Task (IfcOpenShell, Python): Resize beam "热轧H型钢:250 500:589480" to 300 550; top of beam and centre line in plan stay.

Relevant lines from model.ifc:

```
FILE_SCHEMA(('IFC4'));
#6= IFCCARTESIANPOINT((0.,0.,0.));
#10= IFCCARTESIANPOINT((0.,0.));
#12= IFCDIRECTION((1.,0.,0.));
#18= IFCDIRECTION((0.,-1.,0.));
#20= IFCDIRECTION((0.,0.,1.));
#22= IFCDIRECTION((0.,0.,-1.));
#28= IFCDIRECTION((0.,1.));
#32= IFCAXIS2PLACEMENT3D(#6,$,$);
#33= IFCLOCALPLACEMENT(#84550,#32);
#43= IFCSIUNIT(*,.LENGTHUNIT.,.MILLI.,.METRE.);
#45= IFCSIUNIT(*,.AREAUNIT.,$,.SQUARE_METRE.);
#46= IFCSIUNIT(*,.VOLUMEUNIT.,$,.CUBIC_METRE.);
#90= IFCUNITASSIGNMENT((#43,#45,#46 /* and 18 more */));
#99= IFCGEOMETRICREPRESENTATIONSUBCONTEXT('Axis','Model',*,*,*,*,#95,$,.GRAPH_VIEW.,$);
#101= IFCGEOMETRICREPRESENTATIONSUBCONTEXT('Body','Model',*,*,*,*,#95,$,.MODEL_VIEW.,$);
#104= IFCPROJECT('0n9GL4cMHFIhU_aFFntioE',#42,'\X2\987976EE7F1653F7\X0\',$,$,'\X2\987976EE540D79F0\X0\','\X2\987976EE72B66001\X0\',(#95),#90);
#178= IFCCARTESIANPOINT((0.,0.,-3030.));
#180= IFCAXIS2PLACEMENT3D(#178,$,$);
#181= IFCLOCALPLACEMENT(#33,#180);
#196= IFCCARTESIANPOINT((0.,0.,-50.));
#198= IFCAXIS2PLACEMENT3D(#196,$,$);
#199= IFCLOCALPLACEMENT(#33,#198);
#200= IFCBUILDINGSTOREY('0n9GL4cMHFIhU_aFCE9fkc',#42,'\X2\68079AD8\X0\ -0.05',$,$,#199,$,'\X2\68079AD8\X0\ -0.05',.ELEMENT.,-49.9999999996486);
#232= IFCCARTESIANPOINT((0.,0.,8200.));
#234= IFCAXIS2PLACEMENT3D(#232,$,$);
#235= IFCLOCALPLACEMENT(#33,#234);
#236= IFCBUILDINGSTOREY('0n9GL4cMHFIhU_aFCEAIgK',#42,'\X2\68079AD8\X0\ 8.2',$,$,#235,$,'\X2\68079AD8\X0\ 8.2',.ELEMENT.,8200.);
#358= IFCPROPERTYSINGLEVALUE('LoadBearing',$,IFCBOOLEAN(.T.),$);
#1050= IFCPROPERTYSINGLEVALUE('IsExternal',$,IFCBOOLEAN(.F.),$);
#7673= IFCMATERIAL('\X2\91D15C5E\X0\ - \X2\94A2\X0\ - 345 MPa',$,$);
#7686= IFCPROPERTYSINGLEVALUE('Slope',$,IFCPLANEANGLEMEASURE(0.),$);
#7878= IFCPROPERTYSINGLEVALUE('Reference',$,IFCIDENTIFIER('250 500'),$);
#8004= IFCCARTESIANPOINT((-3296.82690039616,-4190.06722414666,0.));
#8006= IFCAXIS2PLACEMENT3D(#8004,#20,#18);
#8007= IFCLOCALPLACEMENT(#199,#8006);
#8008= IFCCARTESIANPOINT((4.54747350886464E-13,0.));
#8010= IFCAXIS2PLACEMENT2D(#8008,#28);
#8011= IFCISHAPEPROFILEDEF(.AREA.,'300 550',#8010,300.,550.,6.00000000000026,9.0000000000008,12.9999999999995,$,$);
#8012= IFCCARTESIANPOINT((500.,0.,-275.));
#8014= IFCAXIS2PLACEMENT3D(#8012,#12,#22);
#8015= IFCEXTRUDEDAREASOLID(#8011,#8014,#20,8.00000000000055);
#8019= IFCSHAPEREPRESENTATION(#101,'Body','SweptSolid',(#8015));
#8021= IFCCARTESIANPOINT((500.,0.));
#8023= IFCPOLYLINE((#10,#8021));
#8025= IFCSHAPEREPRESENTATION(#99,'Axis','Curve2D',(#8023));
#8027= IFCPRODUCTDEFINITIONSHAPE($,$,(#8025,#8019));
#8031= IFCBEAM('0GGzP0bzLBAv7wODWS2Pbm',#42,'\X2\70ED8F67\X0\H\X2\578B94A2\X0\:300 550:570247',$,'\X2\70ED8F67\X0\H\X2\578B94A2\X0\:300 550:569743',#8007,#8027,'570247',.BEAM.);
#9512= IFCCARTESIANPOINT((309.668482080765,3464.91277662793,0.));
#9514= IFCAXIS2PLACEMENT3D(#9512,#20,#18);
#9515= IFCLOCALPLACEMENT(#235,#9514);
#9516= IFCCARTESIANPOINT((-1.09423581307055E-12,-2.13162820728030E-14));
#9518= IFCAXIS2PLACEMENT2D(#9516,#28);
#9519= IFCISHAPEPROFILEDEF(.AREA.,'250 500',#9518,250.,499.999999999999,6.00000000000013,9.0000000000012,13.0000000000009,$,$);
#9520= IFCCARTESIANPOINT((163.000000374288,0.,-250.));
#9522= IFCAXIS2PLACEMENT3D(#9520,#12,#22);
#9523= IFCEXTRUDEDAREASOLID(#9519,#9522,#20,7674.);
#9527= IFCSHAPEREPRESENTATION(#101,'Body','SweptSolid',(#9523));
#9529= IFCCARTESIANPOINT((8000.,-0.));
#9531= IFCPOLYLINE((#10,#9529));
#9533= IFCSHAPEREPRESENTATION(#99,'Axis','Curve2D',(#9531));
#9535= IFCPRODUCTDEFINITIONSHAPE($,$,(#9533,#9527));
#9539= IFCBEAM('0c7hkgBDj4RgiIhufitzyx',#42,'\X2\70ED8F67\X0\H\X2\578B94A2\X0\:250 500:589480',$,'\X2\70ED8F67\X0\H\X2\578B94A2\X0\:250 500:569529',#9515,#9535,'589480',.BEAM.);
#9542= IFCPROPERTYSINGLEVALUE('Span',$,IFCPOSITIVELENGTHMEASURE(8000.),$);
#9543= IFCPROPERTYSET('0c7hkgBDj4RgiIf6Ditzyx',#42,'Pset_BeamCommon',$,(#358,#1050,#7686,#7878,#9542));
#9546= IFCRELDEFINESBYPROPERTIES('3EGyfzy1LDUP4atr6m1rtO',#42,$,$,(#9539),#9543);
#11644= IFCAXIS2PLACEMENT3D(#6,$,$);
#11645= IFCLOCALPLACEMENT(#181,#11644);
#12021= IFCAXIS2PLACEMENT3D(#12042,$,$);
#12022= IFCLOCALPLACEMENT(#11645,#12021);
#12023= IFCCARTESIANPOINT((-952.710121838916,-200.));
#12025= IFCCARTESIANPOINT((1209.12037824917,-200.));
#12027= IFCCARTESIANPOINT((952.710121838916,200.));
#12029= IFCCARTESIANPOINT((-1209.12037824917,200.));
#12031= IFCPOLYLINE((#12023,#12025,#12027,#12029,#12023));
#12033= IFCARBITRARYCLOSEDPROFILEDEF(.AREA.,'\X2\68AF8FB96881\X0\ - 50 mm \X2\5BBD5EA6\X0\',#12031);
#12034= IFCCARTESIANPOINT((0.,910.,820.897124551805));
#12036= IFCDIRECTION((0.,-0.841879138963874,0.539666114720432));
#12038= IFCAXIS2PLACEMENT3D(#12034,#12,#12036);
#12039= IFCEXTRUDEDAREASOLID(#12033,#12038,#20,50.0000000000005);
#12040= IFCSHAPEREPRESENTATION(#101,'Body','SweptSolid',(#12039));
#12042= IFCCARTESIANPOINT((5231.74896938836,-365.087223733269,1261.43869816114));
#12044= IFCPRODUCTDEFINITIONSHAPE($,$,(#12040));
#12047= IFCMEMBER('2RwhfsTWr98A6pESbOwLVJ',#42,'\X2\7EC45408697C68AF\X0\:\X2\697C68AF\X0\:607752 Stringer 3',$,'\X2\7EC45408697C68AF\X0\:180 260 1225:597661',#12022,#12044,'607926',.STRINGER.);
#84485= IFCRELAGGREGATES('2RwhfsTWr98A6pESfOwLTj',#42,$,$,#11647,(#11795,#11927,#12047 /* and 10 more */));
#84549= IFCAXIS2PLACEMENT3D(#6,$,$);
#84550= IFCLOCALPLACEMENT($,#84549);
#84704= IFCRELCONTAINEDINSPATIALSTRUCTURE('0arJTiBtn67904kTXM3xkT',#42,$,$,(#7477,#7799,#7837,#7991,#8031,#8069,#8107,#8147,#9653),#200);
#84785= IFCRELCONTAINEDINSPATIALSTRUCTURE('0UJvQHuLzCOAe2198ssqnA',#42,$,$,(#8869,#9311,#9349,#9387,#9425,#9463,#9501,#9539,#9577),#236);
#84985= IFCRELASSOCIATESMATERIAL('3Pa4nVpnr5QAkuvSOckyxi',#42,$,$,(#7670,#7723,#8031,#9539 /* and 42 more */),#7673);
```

```python
import ifcopenshell
import ifcopenshell.api.pset
import ifcopenshell.util.element
import ifcopenshell.util.representation

model = ifcopenshell.open("model.ifc")

member = model.by_guid("0c7hkgBDj4RgiIhufitzyx")
source = next(p for p in model.by_type("IfcIShapeProfileDef") if p.ProfileName == "300 550")

body = ifcopenshell.util.representation.get_representation(member, "Model", "Body")
solid = body.Items[0]
old_profile = solid.SweptArea

# Copy the section's sizes but keep this member's own profile position.
profile = ifcopenshell.util.element.copy(model, source)
# Profiles are centred, so shift by half the change in depth to hold the top.
shift = (old_profile.OverallDepth - profile.OverallDepth) / 2
x, y = old_profile.Position.Location.Coordinates
up = (-1.0, 0.0)  # upwards, in the solid's own plane
location = model.createIfcCartesianPoint((x + up[0] * shift, y + up[1] * shift))
profile.Position = model.createIfcAxis2Placement2D(location, old_profile.Position.RefDirection)
solid.SweptArea = profile
if not model.get_total_inverses(old_profile):
    ifcopenshell.util.element.remove_deep2(model, old_profile)
member.Name = member.Name.replace("250 500", "300 550")
member.ObjectType = member.ObjectType.replace("250 500", "300 550")
pset = model.by_id(ifcopenshell.util.element.get_pset(member, "Pset_BeamCommon", should_inherit=False)["id"])
ifcopenshell.api.pset.edit_pset(model, pset=pset, properties={"Reference": "300 550"})

print(solid.SweptArea)

model.write("model_updated.ifc")
```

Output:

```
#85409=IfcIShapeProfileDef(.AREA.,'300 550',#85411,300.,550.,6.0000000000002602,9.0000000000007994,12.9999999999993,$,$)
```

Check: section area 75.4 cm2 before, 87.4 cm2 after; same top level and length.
